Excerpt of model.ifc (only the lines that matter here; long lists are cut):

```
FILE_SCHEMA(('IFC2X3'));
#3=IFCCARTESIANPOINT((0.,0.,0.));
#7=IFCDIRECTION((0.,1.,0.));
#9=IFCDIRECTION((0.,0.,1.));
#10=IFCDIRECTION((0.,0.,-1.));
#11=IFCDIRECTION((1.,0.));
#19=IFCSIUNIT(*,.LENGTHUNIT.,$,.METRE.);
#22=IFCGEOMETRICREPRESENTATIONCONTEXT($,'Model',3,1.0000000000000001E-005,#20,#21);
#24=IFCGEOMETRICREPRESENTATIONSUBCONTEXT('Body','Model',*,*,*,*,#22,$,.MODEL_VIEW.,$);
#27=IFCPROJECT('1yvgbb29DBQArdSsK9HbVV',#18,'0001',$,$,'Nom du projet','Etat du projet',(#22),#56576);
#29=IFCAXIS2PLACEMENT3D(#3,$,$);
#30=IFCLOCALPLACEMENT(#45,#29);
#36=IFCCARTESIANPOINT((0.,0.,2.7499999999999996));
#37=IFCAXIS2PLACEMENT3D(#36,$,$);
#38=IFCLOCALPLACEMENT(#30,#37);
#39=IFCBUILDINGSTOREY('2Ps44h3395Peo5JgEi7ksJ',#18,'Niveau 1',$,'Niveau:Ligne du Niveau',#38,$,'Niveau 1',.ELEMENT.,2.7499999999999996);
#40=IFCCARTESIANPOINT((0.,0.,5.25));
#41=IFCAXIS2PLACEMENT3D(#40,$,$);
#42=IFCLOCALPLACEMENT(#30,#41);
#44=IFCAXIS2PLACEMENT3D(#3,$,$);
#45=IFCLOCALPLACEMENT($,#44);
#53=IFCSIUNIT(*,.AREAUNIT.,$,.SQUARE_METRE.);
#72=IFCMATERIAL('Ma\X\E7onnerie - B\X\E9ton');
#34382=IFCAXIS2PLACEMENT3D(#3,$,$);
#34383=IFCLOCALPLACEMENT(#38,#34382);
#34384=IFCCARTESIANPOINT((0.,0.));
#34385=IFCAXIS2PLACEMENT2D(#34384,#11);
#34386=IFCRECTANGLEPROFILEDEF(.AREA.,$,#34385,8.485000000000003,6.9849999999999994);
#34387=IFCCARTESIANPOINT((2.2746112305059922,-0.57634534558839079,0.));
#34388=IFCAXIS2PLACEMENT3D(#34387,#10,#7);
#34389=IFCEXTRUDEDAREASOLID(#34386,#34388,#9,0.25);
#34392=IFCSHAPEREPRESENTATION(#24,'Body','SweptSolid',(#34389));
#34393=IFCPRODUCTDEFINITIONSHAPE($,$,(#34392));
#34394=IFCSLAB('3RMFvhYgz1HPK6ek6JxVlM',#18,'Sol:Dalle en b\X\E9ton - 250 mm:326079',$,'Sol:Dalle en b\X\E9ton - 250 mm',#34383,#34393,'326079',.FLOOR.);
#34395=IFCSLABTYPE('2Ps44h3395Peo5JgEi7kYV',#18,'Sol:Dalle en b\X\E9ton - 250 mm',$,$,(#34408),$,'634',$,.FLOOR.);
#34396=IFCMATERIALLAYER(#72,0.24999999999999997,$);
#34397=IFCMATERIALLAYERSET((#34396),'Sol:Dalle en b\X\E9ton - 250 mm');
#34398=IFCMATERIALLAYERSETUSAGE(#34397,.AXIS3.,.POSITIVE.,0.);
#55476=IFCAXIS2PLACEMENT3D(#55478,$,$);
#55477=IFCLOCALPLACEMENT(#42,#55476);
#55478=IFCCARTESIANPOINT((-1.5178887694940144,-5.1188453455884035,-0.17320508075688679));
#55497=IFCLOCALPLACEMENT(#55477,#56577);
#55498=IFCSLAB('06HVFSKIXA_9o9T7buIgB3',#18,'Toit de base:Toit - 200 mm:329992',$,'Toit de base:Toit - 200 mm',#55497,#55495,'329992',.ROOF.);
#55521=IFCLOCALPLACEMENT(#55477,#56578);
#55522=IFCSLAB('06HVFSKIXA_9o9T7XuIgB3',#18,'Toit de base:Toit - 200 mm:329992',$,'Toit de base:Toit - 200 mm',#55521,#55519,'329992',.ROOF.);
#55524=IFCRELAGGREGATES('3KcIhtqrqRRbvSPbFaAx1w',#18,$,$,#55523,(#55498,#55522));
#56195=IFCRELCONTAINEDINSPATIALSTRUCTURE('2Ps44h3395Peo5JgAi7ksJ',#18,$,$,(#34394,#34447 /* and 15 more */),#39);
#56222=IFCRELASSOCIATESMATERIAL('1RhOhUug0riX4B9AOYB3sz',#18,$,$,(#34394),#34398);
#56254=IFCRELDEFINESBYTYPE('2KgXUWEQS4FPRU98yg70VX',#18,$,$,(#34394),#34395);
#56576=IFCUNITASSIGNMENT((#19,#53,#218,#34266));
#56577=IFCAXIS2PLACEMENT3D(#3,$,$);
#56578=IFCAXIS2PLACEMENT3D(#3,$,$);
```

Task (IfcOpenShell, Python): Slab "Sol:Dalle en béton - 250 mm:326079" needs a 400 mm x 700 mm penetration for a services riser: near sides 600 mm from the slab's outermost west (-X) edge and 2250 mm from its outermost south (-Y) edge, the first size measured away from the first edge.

```python
import numpy as np
import ifcopenshell
import ifcopenshell.api.feature
import ifcopenshell.api.geometry
import ifcopenshell.api.root
import ifcopenshell.geom
import ifcopenshell.util.placement
import ifcopenshell.util.representation
import ifcopenshell.util.shape
import ifcopenshell.util.unit

model = ifcopenshell.open("model.ifc")
unit_scale = ifcopenshell.util.unit.calculate_unit_scale(model)
settings = ifcopenshell.geom.settings()


def volume(element):
    """Net volume in cubic metres, openings subtracted."""
    shape = ifcopenshell.geom.create_shape(settings, element)
    return ifcopenshell.util.shape.get_volume(shape.geometry)


slab = model.by_id(34394)
before = volume(slab)

# Extent in the slab's own axes, in metres. The edges named are its -X and -Y sides.
slab_shape = ifcopenshell.geom.create_shape(settings, slab)
vertices = ifcopenshell.util.shape.get_vertices(slab_shape.geometry)
x_min, y_min, bottom = vertices.min(axis=0)
top = vertices[:, 2].max()

opening = ifcopenshell.api.root.create_entity(model, ifc_class="IfcOpeningElement", name="Services riser opening")
context = ifcopenshell.util.representation.get_context(model, "Model", "Body", "MODEL_VIEW")
width, depth = 0.4, 0.7
outline = [(0.0, 0.0), (width, 0.0), (width, depth), (0.0, depth), (0.0, 0.0)]
# Overshoot both faces by 50 mm so the cut is clean.
shape = ifcopenshell.api.geometry.add_slab_representation(
    model, context=context, depth=top - bottom + 0.1, polyline=outline
)
ifcopenshell.api.geometry.assign_representation(model, product=opening, representation=shape)

matrix = ifcopenshell.util.placement.get_local_placement(slab.ObjectPlacement)
matrix[:, 3] = matrix @ np.append(np.array([x_min + 0.6, y_min + 2.25, bottom - 0.05]) / unit_scale, 1.0)
ifcopenshell.api.geometry.edit_object_placement(model, product=opening, matrix=matrix, is_si=False)
ifcopenshell.api.feature.add_feature(model, feature=opening, element=slab)

after = volume(slab)

print(f"slab volume {before:.3f} -> {after:.3f} m3")

model.write("model_v2.ifc")
```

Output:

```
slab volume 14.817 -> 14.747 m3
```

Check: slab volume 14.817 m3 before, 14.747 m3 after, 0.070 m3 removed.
